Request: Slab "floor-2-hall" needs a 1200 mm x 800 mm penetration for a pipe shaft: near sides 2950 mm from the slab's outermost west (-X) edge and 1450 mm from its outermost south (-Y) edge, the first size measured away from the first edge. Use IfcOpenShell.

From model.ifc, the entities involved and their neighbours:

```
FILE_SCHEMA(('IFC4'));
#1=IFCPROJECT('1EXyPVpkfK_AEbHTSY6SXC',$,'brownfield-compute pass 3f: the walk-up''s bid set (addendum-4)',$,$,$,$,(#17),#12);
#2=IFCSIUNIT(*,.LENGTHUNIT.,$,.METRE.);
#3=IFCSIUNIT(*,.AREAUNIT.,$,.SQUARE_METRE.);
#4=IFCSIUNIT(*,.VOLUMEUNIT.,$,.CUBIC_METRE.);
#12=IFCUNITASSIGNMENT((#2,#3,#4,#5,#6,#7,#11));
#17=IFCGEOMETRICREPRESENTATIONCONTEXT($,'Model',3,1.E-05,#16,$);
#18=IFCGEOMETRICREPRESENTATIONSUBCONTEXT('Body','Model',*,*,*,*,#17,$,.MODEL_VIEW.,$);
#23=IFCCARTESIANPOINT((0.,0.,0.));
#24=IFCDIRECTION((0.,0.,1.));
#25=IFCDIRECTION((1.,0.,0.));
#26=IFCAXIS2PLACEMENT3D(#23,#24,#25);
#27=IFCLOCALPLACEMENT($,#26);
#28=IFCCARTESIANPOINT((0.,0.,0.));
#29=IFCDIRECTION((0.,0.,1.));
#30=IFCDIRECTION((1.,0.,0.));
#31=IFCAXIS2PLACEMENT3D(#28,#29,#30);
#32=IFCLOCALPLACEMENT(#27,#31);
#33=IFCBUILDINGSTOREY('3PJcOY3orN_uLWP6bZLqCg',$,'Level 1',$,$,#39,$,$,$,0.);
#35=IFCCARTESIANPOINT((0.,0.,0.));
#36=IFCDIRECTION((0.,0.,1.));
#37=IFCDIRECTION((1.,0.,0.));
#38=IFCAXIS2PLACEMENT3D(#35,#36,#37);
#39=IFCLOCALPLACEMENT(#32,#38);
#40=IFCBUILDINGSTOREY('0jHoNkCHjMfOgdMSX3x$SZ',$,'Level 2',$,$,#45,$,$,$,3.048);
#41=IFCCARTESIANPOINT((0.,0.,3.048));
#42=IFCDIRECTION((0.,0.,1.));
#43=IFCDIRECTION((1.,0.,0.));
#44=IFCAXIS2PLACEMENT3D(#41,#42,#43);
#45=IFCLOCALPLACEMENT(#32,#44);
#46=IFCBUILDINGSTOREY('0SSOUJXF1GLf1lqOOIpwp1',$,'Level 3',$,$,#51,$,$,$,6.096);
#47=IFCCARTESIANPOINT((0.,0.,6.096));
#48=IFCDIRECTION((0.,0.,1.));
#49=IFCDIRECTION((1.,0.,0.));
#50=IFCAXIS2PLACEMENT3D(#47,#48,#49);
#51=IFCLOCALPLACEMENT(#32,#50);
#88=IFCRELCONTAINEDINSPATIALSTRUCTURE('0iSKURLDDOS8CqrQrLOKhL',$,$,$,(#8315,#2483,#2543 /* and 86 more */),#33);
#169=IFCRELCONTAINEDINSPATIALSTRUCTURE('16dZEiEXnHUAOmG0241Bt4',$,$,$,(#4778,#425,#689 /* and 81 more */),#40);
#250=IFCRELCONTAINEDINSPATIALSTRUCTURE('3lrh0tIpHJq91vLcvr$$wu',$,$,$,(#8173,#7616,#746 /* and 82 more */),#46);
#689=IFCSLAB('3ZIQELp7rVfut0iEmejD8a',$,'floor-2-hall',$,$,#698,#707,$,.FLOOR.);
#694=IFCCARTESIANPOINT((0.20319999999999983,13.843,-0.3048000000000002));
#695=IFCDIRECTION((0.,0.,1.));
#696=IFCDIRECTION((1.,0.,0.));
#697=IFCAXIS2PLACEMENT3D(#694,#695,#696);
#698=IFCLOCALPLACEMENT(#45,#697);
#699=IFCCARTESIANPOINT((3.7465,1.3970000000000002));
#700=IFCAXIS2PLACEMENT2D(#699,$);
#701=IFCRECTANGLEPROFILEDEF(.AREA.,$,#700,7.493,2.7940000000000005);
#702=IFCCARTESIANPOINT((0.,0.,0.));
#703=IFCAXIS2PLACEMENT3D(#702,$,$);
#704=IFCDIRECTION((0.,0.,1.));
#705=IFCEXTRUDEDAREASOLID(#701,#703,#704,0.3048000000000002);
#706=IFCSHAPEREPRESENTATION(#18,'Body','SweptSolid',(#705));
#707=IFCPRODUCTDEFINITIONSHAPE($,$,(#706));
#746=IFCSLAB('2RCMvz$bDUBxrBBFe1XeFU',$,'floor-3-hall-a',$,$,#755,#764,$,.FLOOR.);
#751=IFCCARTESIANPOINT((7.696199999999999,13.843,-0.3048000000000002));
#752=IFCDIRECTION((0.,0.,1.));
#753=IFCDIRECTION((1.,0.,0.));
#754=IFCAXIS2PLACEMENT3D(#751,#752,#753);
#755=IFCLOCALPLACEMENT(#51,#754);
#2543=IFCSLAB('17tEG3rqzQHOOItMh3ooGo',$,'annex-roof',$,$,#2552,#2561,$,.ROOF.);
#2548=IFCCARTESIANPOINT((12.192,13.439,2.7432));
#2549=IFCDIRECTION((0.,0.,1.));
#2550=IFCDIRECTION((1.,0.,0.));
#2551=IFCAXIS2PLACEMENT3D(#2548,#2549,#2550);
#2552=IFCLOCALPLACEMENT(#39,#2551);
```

```python
import numpy as np
import ifcopenshell
import ifcopenshell.api.feature
import ifcopenshell.api.geometry
import ifcopenshell.api.root
import ifcopenshell.geom
import ifcopenshell.util.placement
import ifcopenshell.util.representation
import ifcopenshell.util.shape
import ifcopenshell.util.unit

model = ifcopenshell.open("model.ifc")
unit_scale = ifcopenshell.util.unit.calculate_unit_scale(model)
settings = ifcopenshell.geom.settings()


def volume(element):
    """Net volume in cubic metres, openings subtracted."""
    shape = ifcopenshell.geom.create_shape(settings, element)
    return ifcopenshell.util.shape.get_volume(shape.geometry)


slab = model.by_guid("3ZIQELp7rVfut0iEmejD8a")
before = volume(slab)

# Extent in the slab's own axes, in metres. The edges named are its -X and -Y sides.
slab_shape = ifcopenshell.geom.create_shape(settings, slab)
vertices = ifcopenshell.util.shape.get_vertices(slab_shape.geometry)
x_min, y_min, bottom = vertices.min(axis=0)
top = vertices[:, 2].max()

opening = ifcopenshell.api.root.create_entity(model, ifc_class="IfcOpeningElement", name="Pipe shaft opening", predefined_type="OPENING")
context = ifcopenshell.util.representation.get_context(model, "Model", "Body", "MODEL_VIEW")
width, depth = 1.2, 0.8
outline = [(0.0, 0.0), (width, 0.0), (width, depth), (0.0, depth), (0.0, 0.0)]
# Overshoot both faces by 50 mm so the cut is clean.
shape = ifcopenshell.api.geometry.add_slab_representation(
    model, context=context, depth=top - bottom + 0.1, polyline=outline
)
ifcopenshell.api.geometry.assign_representation(model, product=opening, representation=shape)

matrix = ifcopenshell.util.placement.get_local_placement(slab.ObjectPlacement)
matrix[:, 3] = matrix @ np.append(np.array([x_min + 2.95, y_min + 1.45, bottom - 0.05]) / unit_scale, 1.0)
ifcopenshell.api.geometry.edit_object_placement(model, product=opening, matrix=matrix, is_si=False)
ifcopenshell.api.feature.add_feature(model, feature=opening, element=slab)

after = volume(slab)

print(f"slab volume {before:.3f} -> {after:.3f} m3")

model.write("model_edited.ifc")
```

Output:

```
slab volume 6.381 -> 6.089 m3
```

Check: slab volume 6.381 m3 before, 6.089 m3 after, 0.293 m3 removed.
